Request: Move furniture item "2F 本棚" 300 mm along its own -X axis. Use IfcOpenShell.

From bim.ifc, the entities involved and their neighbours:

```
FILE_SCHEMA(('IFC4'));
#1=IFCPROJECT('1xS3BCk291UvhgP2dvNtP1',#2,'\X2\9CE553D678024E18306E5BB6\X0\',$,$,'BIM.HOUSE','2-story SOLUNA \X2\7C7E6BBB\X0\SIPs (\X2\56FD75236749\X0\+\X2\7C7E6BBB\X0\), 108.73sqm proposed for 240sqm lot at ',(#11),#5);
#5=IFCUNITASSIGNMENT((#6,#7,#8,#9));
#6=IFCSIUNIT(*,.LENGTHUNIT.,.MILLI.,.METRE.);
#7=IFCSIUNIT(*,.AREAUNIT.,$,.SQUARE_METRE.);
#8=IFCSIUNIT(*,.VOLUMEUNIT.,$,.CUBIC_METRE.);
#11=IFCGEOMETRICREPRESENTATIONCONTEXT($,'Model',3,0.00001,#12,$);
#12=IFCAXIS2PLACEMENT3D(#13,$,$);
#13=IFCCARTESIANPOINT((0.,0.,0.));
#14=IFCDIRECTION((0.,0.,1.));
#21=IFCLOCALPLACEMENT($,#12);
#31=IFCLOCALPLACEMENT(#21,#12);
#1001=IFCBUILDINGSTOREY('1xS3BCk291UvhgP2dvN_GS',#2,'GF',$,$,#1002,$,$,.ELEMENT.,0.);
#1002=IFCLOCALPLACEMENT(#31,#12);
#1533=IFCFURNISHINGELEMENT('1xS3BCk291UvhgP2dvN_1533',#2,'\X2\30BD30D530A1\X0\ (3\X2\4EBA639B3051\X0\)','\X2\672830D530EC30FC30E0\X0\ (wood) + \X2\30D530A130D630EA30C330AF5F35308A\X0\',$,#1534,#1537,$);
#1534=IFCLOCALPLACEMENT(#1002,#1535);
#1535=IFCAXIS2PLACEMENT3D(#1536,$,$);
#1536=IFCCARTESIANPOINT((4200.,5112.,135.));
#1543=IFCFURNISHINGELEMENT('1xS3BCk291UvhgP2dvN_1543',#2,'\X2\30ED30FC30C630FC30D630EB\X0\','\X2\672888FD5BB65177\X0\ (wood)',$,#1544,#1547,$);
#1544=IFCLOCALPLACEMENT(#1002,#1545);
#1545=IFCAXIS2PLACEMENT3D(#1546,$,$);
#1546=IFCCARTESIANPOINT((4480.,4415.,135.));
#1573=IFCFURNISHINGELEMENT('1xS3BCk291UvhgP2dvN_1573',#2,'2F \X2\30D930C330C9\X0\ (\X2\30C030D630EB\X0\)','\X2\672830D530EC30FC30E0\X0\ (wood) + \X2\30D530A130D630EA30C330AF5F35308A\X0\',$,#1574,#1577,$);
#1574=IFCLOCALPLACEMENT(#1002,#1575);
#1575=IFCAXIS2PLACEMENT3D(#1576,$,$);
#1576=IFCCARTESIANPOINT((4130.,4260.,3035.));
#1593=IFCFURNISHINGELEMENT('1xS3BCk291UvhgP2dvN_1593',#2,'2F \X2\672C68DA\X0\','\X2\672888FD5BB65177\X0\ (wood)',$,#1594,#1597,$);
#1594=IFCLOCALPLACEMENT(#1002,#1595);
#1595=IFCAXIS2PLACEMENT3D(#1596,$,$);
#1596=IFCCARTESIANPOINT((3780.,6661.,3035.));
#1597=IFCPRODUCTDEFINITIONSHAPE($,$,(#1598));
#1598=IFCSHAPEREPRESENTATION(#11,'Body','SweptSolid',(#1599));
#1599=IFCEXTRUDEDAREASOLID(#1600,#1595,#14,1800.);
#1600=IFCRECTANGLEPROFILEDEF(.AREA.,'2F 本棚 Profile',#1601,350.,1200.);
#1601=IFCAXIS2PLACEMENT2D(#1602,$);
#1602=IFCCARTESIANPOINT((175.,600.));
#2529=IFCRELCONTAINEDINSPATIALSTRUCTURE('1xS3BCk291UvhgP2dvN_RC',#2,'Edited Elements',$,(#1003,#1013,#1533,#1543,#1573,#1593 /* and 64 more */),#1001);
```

```python
import ifcopenshell
import ifcopenshell.api.geometry
import ifcopenshell.util.placement

model = ifcopenshell.open("bim.ifc")

item = model.by_id(1593)
matrix = ifcopenshell.util.placement.get_local_placement(item.ObjectPlacement)
matrix[:3, 3] -= matrix[:3, 0] * 300.0
ifcopenshell.api.geometry.edit_object_placement(model, product=item, matrix=matrix, is_si=False)

print(ifcopenshell.util.placement.get_local_placement(item.ObjectPlacement).round(3) + 0.0)

model.write("bim_v2.ifc")
```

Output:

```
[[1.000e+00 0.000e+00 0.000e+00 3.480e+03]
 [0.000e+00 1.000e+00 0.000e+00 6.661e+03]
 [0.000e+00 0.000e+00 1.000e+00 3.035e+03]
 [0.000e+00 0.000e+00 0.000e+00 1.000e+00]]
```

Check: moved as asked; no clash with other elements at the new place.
